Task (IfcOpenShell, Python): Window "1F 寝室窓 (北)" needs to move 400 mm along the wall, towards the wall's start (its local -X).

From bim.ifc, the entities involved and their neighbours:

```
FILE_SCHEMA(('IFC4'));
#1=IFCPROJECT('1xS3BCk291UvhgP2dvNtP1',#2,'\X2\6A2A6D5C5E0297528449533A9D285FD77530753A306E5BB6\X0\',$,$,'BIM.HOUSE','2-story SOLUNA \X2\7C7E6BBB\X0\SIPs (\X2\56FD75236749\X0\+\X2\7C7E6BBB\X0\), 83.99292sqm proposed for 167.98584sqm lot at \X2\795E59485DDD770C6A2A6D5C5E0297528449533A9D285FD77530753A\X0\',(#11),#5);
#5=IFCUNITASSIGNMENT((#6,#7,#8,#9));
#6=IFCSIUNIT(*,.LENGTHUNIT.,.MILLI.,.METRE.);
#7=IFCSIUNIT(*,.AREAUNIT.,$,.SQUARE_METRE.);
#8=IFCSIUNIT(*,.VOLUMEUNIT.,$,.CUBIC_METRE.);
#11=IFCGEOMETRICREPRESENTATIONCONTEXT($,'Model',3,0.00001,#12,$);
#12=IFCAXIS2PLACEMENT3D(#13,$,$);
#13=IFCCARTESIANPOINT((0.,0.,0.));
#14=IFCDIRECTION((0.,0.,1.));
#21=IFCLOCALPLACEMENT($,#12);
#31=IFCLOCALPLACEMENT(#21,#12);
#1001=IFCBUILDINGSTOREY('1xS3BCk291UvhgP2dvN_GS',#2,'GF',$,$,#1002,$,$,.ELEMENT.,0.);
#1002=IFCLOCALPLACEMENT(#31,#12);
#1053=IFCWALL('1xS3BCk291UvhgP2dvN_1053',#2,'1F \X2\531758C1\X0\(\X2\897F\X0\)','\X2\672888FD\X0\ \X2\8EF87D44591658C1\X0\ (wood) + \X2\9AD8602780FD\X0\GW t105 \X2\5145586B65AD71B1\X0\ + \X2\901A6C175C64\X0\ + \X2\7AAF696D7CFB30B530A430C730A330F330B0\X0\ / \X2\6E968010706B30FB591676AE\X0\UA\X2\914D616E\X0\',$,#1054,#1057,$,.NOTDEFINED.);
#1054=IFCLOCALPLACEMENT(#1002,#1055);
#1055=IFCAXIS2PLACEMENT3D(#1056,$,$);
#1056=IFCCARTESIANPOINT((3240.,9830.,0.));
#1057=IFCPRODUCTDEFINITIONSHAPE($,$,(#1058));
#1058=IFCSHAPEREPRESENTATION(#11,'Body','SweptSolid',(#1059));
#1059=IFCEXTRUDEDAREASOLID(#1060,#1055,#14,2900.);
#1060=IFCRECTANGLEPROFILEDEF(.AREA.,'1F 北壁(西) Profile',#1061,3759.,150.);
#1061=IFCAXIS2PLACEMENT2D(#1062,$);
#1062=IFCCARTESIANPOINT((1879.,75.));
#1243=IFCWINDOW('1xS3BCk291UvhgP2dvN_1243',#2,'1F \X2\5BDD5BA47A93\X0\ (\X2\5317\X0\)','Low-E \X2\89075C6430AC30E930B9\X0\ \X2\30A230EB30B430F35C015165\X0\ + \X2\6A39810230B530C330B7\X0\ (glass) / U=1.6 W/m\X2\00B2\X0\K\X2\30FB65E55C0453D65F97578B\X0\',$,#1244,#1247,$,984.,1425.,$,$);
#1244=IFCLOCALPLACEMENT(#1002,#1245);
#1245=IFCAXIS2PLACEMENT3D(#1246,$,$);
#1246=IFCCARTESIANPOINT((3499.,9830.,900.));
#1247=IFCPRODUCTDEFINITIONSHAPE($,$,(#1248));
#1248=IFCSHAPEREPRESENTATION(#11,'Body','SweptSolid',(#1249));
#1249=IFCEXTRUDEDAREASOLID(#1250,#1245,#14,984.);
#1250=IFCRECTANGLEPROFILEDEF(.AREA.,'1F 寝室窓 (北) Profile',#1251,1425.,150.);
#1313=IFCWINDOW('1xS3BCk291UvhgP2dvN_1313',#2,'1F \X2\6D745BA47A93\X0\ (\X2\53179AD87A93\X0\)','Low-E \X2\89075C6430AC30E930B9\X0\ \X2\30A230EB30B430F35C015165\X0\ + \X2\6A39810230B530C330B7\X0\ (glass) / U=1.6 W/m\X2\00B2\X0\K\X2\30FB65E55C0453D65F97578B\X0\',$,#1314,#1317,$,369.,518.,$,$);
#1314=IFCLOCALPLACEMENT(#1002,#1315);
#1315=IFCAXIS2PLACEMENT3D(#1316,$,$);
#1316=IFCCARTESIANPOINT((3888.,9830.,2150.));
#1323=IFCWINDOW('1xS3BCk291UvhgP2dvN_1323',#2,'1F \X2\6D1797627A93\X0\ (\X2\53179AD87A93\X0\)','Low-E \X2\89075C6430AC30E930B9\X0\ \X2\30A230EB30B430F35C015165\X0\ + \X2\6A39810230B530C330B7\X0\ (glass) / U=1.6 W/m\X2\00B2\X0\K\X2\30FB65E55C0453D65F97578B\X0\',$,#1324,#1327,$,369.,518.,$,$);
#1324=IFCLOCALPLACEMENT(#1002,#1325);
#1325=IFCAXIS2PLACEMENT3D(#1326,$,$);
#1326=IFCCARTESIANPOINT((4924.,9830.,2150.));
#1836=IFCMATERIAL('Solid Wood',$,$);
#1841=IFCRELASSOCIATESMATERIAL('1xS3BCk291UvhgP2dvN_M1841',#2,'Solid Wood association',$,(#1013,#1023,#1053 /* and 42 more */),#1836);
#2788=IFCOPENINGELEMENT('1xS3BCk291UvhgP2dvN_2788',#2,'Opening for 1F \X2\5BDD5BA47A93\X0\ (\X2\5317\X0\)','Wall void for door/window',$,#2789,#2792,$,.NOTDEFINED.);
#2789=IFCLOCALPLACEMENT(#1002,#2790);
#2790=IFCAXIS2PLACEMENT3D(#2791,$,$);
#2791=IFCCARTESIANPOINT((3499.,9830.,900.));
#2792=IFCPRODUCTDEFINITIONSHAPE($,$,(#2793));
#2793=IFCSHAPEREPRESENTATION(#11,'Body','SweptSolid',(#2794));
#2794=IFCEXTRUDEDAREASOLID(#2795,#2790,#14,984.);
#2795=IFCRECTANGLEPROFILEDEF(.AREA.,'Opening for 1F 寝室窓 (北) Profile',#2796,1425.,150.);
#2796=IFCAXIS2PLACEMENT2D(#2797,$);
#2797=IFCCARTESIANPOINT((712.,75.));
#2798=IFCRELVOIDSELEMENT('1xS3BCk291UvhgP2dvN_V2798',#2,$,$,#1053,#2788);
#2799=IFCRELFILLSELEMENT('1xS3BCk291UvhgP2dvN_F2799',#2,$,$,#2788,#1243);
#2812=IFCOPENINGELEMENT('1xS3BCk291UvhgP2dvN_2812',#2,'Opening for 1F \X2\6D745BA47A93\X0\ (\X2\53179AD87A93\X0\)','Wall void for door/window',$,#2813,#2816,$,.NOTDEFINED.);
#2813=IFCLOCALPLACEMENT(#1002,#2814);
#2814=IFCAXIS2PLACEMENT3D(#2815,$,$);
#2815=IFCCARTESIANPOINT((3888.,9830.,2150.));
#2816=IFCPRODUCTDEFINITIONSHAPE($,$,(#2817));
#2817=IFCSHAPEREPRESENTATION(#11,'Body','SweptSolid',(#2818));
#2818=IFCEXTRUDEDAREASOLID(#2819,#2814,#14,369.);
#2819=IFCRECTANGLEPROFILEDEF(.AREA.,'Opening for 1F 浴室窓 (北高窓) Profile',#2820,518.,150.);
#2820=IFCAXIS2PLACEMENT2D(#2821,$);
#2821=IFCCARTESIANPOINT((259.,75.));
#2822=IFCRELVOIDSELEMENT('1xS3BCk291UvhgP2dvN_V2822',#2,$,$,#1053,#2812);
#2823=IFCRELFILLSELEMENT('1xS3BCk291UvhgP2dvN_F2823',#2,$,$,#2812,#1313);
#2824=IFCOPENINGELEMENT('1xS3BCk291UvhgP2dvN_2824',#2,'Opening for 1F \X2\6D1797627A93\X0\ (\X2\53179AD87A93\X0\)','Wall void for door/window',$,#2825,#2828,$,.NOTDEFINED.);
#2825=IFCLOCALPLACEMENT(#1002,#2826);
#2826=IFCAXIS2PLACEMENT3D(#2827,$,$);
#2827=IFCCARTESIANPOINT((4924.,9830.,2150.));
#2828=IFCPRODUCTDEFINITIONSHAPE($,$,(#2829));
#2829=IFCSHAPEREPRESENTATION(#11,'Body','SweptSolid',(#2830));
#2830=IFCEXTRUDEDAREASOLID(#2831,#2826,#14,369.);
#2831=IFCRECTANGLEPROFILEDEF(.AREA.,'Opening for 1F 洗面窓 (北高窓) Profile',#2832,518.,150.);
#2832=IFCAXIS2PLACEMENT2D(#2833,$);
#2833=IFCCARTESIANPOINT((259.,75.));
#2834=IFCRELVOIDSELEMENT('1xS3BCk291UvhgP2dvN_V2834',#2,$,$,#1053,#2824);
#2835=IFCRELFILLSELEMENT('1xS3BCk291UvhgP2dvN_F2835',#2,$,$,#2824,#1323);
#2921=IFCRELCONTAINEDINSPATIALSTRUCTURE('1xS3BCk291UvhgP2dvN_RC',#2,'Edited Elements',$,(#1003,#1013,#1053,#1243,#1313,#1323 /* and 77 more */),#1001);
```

```python
import ifcopenshell
import ifcopenshell.api.geometry
import ifcopenshell.util.placement

model = ifcopenshell.open("bim.ifc")

window = model.by_guid("1xS3BCk291UvhgP2dvN_1243")
opening = window.FillsVoids[0].RelatingOpeningElement
wall = opening.VoidsElements[0].RelatingBuildingElement

wall_matrix = ifcopenshell.util.placement.get_local_placement(wall.ObjectPlacement)
shift = wall_matrix[:3, 0] * -400.0
before = ifcopenshell.util.placement.get_local_placement(window.ObjectPlacement)[:3, 3].copy()

# The window is not placed relative to its opening, so move both.
for product in (opening, window):
    matrix = ifcopenshell.util.placement.get_local_placement(product.ObjectPlacement)
    matrix[:3, 3] += shift
    ifcopenshell.api.geometry.edit_object_placement(model, product=product, matrix=matrix, is_si=False)

after = ifcopenshell.util.placement.get_local_placement(window.ObjectPlacement)[:3, 3]
print("window moved by", (after - before).round(3) + 0.0)

model.write("bim_v2.ifc")
```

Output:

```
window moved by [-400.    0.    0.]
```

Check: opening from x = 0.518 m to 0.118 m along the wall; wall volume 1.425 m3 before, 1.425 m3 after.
